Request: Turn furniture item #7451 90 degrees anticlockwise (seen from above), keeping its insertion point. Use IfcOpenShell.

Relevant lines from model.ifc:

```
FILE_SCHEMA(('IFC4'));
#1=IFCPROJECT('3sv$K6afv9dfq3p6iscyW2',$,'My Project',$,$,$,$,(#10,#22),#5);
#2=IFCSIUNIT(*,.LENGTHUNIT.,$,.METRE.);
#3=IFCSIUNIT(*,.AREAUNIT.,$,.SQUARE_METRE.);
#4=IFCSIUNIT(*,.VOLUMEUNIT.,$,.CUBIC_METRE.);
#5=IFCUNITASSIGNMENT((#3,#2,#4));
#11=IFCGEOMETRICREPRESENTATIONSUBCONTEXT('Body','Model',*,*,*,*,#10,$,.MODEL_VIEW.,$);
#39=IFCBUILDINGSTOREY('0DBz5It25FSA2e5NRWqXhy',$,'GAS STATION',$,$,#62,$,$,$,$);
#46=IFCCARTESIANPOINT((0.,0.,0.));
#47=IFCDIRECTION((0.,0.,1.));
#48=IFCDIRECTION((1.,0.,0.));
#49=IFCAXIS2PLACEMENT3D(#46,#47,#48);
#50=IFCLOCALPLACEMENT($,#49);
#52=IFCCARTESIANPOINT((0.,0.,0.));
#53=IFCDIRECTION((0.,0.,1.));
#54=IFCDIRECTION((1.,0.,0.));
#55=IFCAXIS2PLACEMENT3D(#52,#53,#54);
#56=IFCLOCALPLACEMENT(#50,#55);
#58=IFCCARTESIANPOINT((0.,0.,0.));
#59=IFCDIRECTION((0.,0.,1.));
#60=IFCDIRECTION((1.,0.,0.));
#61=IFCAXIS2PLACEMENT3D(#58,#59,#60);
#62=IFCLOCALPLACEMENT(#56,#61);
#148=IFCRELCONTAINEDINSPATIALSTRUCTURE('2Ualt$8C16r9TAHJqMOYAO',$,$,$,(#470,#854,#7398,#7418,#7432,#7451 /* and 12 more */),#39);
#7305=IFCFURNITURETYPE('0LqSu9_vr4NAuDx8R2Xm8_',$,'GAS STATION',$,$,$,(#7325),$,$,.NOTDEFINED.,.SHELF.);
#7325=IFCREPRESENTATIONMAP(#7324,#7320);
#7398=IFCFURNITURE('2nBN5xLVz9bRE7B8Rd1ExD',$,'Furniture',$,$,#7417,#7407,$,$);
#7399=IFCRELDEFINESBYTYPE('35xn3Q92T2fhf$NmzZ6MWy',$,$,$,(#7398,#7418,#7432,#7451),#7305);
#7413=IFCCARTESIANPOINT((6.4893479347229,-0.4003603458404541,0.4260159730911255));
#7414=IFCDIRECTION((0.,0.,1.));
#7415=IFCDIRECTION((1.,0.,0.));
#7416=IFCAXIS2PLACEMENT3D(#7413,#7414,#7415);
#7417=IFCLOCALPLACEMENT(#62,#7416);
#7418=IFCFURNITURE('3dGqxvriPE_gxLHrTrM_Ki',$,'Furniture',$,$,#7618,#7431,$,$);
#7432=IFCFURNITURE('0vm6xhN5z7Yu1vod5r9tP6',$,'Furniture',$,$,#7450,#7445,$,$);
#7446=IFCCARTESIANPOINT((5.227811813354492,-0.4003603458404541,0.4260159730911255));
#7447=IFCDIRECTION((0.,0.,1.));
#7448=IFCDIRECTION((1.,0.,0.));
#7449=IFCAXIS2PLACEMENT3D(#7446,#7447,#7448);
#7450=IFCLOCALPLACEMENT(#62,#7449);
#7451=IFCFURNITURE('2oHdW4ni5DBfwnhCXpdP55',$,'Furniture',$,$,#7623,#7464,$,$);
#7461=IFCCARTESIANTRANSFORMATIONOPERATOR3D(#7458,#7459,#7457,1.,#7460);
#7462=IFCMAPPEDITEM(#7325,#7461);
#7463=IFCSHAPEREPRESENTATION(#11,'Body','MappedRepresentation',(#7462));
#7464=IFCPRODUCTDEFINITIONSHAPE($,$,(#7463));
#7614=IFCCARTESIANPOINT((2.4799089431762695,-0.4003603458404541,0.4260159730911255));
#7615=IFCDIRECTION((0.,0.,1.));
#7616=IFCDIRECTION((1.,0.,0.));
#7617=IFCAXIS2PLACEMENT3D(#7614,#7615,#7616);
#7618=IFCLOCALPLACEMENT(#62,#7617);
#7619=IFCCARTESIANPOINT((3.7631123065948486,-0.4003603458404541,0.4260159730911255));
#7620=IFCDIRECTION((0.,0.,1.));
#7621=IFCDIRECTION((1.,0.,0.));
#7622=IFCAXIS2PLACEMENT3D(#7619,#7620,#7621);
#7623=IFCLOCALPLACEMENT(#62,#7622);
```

```python
import ifcopenshell
import ifcopenshell.api.geometry
import ifcopenshell.util.placement

model = ifcopenshell.open("model.ifc")

item = model.by_id(7451)
matrix = ifcopenshell.util.placement.get_local_placement(item.ObjectPlacement)
matrix = matrix @ ifcopenshell.util.placement.rotation(90, "Z")
ifcopenshell.api.geometry.edit_object_placement(model, product=item, matrix=matrix, is_si=False)

print(ifcopenshell.util.placement.get_local_placement(item.ObjectPlacement).round(3) + 0.0)

model.write("model_v2.ifc")
```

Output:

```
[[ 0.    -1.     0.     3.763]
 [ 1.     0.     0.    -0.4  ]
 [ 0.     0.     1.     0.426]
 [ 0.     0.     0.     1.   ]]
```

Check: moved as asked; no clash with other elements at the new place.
